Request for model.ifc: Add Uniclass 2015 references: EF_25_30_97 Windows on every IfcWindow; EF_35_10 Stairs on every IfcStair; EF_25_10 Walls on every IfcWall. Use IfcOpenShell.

First a look at what the model holds.

```python
import ifcopenshell

model = ifcopenshell.open("model.ifc")
print(model.schema)
print("classifications:", [c.Name for c in model.by_type("IfcClassification")])
for ifc_class in ("IfcDoor", "IfcRoof", "IfcStair", "IfcWall", "IfcWindow"):
    print(ifc_class, len(model.by_type(ifc_class)))
```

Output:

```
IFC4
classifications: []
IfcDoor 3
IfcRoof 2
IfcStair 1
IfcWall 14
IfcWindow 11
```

```python
import ifcopenshell
import ifcopenshell.api.classification

model = ifcopenshell.open("model.ifc")

system = ifcopenshell.api.classification.add_classification(model, classification="Uniclass 2015")

codes = {
    "IfcWindow": ("EF_25_30_97", "Windows"),
    "IfcStair": ("EF_35_10", "Stairs"),
    "IfcWall": ("EF_25_10", "Walls"),
}
for ifc_class, (code, name) in codes.items():
    products = model.by_type(ifc_class)
    ifcopenshell.api.classification.add_reference(
        model, products=products, classification=system, identification=code, name=name
    )
    print(code, len(products))

model.write("model_updated.ifc")
```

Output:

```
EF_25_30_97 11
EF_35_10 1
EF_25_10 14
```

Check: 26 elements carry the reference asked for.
